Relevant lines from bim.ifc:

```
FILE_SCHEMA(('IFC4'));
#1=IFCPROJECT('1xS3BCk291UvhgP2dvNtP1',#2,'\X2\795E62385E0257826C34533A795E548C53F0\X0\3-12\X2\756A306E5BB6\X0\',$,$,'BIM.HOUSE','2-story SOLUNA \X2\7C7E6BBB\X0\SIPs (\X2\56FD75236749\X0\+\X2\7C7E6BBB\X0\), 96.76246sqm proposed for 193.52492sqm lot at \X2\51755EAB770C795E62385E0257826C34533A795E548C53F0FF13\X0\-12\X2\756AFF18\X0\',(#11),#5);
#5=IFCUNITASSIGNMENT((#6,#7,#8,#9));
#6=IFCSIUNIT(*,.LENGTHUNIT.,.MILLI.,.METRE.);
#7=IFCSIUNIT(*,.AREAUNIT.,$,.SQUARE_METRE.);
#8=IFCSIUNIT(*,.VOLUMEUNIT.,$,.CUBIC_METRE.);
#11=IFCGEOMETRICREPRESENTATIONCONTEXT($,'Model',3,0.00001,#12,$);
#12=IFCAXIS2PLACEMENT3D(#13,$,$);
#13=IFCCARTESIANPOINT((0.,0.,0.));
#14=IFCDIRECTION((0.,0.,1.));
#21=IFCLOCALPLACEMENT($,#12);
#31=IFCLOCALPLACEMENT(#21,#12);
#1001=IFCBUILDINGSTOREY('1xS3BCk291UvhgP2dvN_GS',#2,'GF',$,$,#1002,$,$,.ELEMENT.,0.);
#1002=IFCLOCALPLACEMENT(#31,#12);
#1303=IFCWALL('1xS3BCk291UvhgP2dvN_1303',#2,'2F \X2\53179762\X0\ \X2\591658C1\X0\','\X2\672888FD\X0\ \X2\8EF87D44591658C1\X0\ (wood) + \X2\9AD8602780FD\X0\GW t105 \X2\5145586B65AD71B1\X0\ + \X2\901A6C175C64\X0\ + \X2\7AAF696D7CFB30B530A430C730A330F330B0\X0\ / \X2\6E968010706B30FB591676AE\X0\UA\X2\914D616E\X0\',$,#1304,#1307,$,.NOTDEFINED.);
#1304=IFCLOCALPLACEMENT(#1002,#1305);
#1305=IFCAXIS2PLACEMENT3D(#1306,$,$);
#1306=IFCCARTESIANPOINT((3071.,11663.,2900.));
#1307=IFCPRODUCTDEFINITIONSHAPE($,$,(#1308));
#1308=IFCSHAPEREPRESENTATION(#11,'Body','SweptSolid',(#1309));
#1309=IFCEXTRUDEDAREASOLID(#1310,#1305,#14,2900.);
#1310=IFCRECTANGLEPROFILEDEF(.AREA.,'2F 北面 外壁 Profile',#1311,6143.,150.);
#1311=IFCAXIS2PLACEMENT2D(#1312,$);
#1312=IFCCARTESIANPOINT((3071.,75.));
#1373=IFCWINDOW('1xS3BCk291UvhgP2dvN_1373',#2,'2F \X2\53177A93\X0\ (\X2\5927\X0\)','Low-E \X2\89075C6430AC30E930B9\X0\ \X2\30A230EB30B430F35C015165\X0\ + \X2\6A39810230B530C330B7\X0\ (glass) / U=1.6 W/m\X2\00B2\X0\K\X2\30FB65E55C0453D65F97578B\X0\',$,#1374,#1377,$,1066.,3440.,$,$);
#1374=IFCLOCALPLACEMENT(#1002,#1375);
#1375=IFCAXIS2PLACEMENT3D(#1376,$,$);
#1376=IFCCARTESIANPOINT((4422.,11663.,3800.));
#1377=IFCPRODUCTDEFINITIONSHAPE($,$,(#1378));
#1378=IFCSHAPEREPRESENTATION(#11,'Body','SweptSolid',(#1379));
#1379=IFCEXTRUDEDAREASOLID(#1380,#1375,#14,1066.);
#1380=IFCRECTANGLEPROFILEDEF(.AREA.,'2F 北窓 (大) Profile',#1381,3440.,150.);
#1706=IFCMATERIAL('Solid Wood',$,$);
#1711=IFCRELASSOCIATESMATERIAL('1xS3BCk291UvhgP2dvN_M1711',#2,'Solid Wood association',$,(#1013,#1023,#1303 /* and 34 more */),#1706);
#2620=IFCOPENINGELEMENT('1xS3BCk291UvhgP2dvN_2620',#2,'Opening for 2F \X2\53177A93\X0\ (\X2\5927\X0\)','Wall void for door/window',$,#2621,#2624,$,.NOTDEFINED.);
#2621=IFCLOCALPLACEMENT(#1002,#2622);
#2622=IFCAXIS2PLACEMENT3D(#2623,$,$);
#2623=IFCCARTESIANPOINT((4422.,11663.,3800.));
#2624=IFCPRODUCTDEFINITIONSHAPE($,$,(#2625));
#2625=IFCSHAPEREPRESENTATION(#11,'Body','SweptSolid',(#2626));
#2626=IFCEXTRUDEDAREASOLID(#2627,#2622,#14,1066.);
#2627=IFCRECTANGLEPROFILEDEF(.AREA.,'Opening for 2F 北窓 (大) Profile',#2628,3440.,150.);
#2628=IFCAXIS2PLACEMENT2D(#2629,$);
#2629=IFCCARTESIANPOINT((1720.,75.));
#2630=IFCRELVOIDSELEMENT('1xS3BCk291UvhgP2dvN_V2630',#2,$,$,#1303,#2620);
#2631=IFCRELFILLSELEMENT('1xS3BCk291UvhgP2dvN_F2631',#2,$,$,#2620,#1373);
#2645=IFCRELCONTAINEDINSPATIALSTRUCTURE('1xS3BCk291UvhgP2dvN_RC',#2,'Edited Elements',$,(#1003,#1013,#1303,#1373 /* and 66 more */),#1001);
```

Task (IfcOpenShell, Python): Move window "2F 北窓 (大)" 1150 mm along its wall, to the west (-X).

```python
import ifcopenshell
import ifcopenshell.api.geometry
import ifcopenshell.util.placement

model = ifcopenshell.open("bim.ifc")

window = model.by_guid("1xS3BCk291UvhgP2dvN_1373")
opening = window.FillsVoids[0].RelatingOpeningElement
wall = opening.VoidsElements[0].RelatingBuildingElement

wall_matrix = ifcopenshell.util.placement.get_local_placement(wall.ObjectPlacement)
shift = wall_matrix[:3, 0] * -1150.0
before = ifcopenshell.util.placement.get_local_placement(window.ObjectPlacement)[:3, 3].copy()

# The window is not placed relative to its opening, so move both.
for product in (opening, window):
    matrix = ifcopenshell.util.placement.get_local_placement(product.ObjectPlacement)
    matrix[:3, 3] += shift
    ifcopenshell.api.geometry.edit_object_placement(model, product=product, matrix=matrix, is_si=False)

after = ifcopenshell.util.placement.get_local_placement(window.ObjectPlacement)[:3, 3]
print("window moved by", (after - before).round(3) + 0.0)

model.write("bim_v2.ifc")
```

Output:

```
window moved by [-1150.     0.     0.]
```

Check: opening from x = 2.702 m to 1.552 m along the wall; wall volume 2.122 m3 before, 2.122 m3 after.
